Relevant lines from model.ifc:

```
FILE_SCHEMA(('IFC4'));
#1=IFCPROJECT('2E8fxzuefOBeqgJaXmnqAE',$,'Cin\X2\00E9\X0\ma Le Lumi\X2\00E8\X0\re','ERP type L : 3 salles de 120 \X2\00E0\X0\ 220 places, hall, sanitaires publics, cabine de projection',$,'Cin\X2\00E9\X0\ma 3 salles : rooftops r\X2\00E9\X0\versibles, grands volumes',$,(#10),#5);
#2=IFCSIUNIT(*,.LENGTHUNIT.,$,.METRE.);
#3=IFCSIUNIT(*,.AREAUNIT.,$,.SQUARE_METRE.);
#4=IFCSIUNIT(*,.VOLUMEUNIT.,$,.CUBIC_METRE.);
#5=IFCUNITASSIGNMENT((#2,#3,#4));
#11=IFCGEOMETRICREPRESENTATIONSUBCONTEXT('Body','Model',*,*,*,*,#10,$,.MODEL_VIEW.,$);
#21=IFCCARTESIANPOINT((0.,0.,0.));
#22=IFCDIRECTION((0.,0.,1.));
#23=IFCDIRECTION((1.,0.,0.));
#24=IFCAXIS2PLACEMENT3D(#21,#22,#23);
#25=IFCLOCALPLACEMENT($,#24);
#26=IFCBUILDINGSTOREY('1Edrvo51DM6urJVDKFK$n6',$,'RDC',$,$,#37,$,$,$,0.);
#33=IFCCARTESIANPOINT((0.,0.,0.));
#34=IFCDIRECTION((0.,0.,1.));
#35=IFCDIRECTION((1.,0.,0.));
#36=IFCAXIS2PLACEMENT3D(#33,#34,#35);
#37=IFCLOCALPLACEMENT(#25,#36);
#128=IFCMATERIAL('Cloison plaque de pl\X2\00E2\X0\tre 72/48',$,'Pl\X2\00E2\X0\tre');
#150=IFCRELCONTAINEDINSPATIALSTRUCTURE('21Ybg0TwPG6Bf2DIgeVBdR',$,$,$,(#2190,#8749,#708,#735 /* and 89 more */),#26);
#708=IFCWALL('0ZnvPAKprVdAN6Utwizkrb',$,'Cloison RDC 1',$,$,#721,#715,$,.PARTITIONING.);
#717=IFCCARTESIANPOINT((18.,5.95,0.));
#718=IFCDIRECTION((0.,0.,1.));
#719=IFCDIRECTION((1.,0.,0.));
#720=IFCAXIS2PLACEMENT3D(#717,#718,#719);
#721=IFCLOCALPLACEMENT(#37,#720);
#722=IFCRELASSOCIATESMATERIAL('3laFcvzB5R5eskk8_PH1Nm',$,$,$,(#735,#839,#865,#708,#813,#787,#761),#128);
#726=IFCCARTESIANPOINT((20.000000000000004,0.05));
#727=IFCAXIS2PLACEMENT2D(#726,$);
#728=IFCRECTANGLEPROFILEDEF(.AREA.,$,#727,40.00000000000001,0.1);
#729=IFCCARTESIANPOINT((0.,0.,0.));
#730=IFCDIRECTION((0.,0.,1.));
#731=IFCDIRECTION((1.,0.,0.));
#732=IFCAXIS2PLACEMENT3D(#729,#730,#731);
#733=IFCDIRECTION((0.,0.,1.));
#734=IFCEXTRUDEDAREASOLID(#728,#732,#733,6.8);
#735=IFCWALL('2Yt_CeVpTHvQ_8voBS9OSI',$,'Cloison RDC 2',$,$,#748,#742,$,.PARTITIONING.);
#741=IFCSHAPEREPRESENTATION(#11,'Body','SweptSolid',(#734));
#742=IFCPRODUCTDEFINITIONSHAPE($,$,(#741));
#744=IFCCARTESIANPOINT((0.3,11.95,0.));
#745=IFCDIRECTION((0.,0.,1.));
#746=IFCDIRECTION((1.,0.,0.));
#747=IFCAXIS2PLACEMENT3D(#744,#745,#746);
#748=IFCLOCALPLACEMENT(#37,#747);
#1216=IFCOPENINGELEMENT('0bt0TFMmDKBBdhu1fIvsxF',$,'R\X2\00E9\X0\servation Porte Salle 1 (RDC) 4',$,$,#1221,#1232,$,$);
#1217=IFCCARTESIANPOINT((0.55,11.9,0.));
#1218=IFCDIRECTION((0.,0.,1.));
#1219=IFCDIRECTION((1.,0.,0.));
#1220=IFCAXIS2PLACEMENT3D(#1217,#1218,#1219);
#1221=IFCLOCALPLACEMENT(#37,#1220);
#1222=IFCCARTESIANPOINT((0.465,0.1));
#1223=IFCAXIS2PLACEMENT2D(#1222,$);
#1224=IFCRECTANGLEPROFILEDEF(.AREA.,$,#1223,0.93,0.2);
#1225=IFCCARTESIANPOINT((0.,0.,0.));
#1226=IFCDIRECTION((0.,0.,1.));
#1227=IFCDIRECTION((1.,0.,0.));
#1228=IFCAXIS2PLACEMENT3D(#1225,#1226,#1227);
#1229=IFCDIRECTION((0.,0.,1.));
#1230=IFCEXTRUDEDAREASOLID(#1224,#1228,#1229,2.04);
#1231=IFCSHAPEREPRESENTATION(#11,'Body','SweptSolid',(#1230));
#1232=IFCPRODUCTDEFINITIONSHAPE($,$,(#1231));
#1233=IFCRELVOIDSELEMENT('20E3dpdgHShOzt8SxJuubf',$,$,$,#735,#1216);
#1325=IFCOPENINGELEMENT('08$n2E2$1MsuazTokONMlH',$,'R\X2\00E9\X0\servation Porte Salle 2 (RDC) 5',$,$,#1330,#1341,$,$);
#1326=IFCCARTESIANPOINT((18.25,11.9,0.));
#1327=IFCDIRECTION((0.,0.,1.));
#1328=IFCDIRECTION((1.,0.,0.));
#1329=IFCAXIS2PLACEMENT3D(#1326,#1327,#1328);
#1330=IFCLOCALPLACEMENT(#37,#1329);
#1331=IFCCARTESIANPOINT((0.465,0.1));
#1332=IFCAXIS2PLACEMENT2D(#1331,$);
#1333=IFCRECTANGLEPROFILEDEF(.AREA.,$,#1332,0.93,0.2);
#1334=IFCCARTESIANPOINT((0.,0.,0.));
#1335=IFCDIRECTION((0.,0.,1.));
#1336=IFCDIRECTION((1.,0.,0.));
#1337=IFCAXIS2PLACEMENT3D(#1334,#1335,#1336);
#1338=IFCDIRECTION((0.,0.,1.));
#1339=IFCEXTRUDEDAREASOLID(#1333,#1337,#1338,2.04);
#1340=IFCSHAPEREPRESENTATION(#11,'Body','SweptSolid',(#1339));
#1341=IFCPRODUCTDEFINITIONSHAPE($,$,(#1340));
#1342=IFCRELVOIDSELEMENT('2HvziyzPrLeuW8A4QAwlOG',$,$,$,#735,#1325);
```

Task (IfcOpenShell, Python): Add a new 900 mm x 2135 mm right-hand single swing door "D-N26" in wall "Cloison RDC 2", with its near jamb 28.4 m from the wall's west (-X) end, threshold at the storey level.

```python
import numpy as np
import ifcopenshell
import ifcopenshell.api.feature
import ifcopenshell.api.geometry
import ifcopenshell.api.root
import ifcopenshell.api.spatial
import ifcopenshell.geom
import ifcopenshell.util.element
import ifcopenshell.util.placement
import ifcopenshell.util.representation
import ifcopenshell.util.shape
import ifcopenshell.util.unit

model = ifcopenshell.open("model.ifc")
unit_scale = ifcopenshell.util.unit.calculate_unit_scale(model)
settings = ifcopenshell.geom.settings()


def volume(element):
    """Net volume in cubic metres, openings subtracted."""
    shape = ifcopenshell.geom.create_shape(settings, element)
    return ifcopenshell.util.shape.get_volume(shape.geometry)


wall = model.by_guid("2Yt_CeVpTHvQ_8voBS9OSI")
storey = ifcopenshell.util.element.get_container(wall, ifc_class="IfcBuildingStorey")
context = ifcopenshell.util.representation.get_context(model, "Model", "Body", "MODEL_VIEW")
before = volume(wall)

width, height, from_end, sill = 0.9, 2.135, 28.4, 0.0  # metres

# The wall runs along its own X axis, and the end named is its -X end.
wall_shape = ifcopenshell.geom.create_shape(settings, wall)
x, y, z = ifcopenshell.util.shape.get_vertices(wall_shape.geometry).T
start = x.min() + from_end
face, thickness = float(y.min()), float(y.max() - y.min())
wall_matrix = ifcopenshell.util.placement.get_local_placement(wall.ObjectPlacement)
level = ifcopenshell.util.placement.get_local_placement(storey.ObjectPlacement)[2, 3]


def in_wall(x, y):
    """Placement at x, y metres in the wall's axes, at sill height."""
    matrix = wall_matrix.copy()
    matrix[:, 3] = wall_matrix @ np.array([x / unit_scale, y / unit_scale, 0.0, 1.0])
    matrix[2, 3] = level + sill / unit_scale
    return matrix


# Opening: a box that overshoots both wall faces by 50 mm.
opening = ifcopenshell.api.root.create_entity(model, ifc_class="IfcOpeningElement", predefined_type="OPENING")
box = ifcopenshell.api.geometry.add_wall_representation(
    model, context=context, length=width, height=height, thickness=thickness + 0.1
)
ifcopenshell.api.geometry.assign_representation(model, product=opening, representation=box)
ifcopenshell.api.geometry.edit_object_placement(model, product=opening, matrix=in_wall(start, face - 0.05), is_si=False)
ifcopenshell.api.feature.add_feature(model, feature=opening, element=wall)

door = ifcopenshell.api.root.create_entity(model, ifc_class="IfcDoor", name="D-N26", predefined_type="DOOR")
door.OverallWidth, door.OverallHeight = width / unit_scale, height / unit_scale
door.OperationType = "SINGLE_SWING_RIGHT"
body = ifcopenshell.api.geometry.add_door_representation(
    model,
    context=context,
    overall_width=door.OverallWidth,
    overall_height=door.OverallHeight,
    operation_type="SINGLE_SWING_RIGHT",
    lining_properties={"LiningDepth": thickness / unit_scale, "ThresholdDepth": thickness / unit_scale},
)
ifcopenshell.api.geometry.assign_representation(model, product=door, representation=body)
ifcopenshell.api.spatial.assign_container(model, products=[door], relating_structure=storey)
ifcopenshell.api.feature.add_filling(model, opening=opening, element=door)

# The lining spans the wall, so the door starts at the wall face.
ifcopenshell.api.geometry.edit_object_placement(model, product=door, matrix=in_wall(start, face), is_si=False)

after = volume(wall)

print(f"wall volume {before:.3f} -> {after:.3f} m3")

model.write("model_edited.ifc")
```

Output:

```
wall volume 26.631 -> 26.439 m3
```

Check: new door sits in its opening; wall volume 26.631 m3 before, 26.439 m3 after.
